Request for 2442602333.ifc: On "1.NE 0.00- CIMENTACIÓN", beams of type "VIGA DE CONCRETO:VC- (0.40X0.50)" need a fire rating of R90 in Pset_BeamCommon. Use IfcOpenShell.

First a look at what the model holds.

```python
import ifcopenshell
import ifcopenshell.util.element

model = ifcopenshell.open("2442602333.ifc")
print(model.schema)
storey = next(s for s in model.by_type("IfcBuildingStorey") if s.Name == "1.NE 0.00- CIMENTACIÓN")
beams = [e for e in ifcopenshell.util.element.get_decomposition(storey) if e.is_a("IfcBeam")]
seen = {}
for e in beams:
    element_type = ifcopenshell.util.element.get_type(e)
    key = (element_type.Name if element_type != e and element_type else None, ifcopenshell.util.element.get_pset(e, "Pset_BeamCommon", "FireRating"))
    seen[key] = seen.get(key, 0) + 1
for (name, value), count in sorted(seen.items(), key=str):
    print(count, "x", name, "|", value)
```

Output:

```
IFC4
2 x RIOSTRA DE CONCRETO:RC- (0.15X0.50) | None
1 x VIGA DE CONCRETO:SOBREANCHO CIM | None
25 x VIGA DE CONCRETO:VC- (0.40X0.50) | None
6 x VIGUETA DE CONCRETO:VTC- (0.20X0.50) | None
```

```python
import ifcopenshell
import ifcopenshell.api.pset
import ifcopenshell.util.element

model = ifcopenshell.open("2442602333.ifc")

storey = next(s for s in model.by_type("IfcBuildingStorey") if s.Name == "1.NE 0.00- CIMENTACIÓN")
beams = [e for e in ifcopenshell.util.element.get_decomposition(storey) if e.is_a("IfcBeam")]

count = 0
for e in beams:
    element_type = ifcopenshell.util.element.get_type(e)
    if element_type in (None, e) or element_type.Name != "VIGA DE CONCRETO:VC- (0.40X0.50)":
        continue
    # add_pset returns the element's existing set when there is one.
    pset = ifcopenshell.api.pset.add_pset(model, product=e, name="Pset_BeamCommon")
    ifcopenshell.api.pset.edit_pset(model, pset=pset, properties={"FireRating": "R90"})
    count += 1

print(count, "beams updated")

model.write("2442602333_v2.ifc")
```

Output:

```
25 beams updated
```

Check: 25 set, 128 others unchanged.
